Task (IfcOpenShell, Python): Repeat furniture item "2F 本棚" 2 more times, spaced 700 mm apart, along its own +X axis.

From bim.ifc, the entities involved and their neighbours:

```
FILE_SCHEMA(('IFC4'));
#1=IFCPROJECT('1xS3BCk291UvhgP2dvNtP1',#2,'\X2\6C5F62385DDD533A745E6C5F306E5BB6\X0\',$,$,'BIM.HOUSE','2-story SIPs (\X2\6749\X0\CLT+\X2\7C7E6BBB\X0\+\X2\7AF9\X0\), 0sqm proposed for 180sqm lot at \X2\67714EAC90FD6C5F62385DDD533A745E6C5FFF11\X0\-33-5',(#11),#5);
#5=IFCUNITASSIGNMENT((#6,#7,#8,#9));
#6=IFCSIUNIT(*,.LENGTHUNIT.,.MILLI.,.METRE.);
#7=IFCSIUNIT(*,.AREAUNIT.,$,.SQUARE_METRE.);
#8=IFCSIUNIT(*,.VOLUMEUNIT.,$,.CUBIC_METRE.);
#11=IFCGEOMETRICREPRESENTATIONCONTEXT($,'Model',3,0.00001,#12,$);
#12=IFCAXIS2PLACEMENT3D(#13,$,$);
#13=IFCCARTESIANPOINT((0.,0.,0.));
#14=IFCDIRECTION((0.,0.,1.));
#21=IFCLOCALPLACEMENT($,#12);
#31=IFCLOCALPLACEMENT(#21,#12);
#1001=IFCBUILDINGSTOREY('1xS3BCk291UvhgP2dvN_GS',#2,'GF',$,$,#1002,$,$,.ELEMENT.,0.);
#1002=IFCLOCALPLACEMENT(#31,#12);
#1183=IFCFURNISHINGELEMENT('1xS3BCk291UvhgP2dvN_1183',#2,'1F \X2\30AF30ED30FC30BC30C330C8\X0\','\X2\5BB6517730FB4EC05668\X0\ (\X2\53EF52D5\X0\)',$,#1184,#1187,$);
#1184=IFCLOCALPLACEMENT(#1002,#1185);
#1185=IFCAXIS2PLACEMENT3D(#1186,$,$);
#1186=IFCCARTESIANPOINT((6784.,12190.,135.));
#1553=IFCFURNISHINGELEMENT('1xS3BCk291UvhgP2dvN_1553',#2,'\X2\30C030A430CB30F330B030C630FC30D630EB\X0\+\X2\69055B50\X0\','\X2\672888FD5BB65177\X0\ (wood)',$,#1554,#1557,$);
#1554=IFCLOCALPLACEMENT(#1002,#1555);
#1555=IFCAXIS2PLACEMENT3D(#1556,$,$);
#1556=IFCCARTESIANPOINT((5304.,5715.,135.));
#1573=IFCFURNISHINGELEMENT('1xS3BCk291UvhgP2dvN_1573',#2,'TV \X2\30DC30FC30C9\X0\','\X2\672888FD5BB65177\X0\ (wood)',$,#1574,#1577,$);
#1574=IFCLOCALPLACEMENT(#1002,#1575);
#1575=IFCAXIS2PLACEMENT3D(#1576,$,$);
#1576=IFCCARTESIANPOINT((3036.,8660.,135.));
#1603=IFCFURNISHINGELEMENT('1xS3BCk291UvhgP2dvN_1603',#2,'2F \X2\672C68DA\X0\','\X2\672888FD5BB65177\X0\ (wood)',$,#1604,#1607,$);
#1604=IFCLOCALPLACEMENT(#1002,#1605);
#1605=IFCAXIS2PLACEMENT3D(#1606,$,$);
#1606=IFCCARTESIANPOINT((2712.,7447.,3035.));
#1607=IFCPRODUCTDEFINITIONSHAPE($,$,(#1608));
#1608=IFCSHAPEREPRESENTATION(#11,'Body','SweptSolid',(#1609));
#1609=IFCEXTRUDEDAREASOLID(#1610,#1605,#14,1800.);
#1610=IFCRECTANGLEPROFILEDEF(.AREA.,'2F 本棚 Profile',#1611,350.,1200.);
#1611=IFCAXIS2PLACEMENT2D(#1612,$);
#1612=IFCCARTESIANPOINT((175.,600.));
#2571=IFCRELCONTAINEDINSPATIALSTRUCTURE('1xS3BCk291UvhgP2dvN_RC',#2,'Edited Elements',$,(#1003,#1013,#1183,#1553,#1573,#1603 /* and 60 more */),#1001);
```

```python
import ifcopenshell
import ifcopenshell.api.geometry
import ifcopenshell.api.root
import ifcopenshell.util.element
import ifcopenshell.util.placement
import ifcopenshell.util.unit

model = ifcopenshell.open("bim.ifc")
unit_scale = ifcopenshell.util.unit.calculate_unit_scale(model)


def reuse_history(source, copy):
    """copy_class also copies each property set's owner history, people and application; keep the originals."""
    for rel in copy.IsDefinedBy:
        if rel.is_a("IfcRelDefinesByProperties") and (history := rel.RelatingPropertyDefinition.OwnerHistory):
            rel.RelatingPropertyDefinition.OwnerHistory = source.OwnerHistory
            ifcopenshell.util.element.remove_deep2(model, history)


source = model.by_id(1603)
base = ifcopenshell.util.placement.get_local_placement(source.ObjectPlacement)
step = base[:3, 0] * 0.7 / unit_scale

for i in range(1, 3):
    copy = ifcopenshell.api.root.copy_class(model, product=source)
    copy.Representation = ifcopenshell.util.element.copy_deep(
        model, source.Representation, exclude=["IfcGeometricRepresentationContext", "IfcRepresentationMap"]
    )
    reuse_history(source, copy)
    matrix = base.copy()
    matrix[:3, 3] += i * step
    print("added at", matrix[:3, 3].round(3) + 0.0)
    ifcopenshell.api.geometry.edit_object_placement(model, product=copy, matrix=matrix, is_si=False)

model.write("bim_edited.ifc")
```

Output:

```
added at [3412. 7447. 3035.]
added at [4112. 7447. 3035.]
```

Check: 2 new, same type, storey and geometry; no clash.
